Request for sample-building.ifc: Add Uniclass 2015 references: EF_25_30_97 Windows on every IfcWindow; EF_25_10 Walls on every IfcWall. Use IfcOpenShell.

First a look at what the model holds.

```python
import ifcopenshell

model = ifcopenshell.open("sample-building.ifc")
print(model.schema)
print("classifications:", [c.Name for c in model.by_type("IfcClassification")])
for ifc_class in ("IfcDoor", "IfcRoof", "IfcStair", "IfcWall", "IfcWindow"):
    print(ifc_class, len(model.by_type(ifc_class)))
```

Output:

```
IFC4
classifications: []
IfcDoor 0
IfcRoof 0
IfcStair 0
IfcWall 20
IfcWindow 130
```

```python
import ifcopenshell
import ifcopenshell.api.classification

model = ifcopenshell.open("sample-building.ifc")

system = ifcopenshell.api.classification.add_classification(model, classification="Uniclass 2015")

codes = {
    "IfcWindow": ("EF_25_30_97", "Windows"),
    "IfcWall": ("EF_25_10", "Walls"),
}
for ifc_class, (code, name) in codes.items():
    products = model.by_type(ifc_class)
    ifcopenshell.api.classification.add_reference(
        model, products=products, classification=system, identification=code, name=name
    )
    print(code, len(products))

model.write("sample-building_v2.ifc")
```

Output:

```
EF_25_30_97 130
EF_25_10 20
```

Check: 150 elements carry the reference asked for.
